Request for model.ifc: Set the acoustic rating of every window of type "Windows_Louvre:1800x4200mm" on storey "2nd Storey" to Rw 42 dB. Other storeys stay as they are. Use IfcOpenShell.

First a look at what the model holds.

```python
import ifcopenshell
import ifcopenshell.util.element

model = ifcopenshell.open("model.ifc")
print(model.schema)
storey = next(s for s in model.by_type("IfcBuildingStorey") if s.Name == "2nd Storey")
windows = [e for e in ifcopenshell.util.element.get_decomposition(storey) if e.is_a("IfcWindow")]
seen = {}
for e in windows:
    element_type = ifcopenshell.util.element.get_type(e)
    key = (element_type.Name if element_type != e and element_type else None, ifcopenshell.util.element.get_pset(e, "Pset_WindowCommon", "AcousticRating"))
    seen[key] = seen.get(key, 0) + 1
for (name, value), count in sorted(seen.items(), key=str):
    print(count, "x", name, "|", value)
```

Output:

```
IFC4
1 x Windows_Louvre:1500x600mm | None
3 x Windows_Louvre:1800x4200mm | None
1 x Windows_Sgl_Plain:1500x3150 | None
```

```python
import ifcopenshell
import ifcopenshell.api.pset
import ifcopenshell.util.element

model = ifcopenshell.open("model.ifc")

storey = next(s for s in model.by_type("IfcBuildingStorey") if s.Name == "2nd Storey")
windows = [e for e in ifcopenshell.util.element.get_decomposition(storey) if e.is_a("IfcWindow")]

count = 0
for e in windows:
    element_type = ifcopenshell.util.element.get_type(e)
    if element_type in (None, e) or element_type.Name != "Windows_Louvre:1800x4200mm":
        continue
    # add_pset returns the element's existing set when there is one.
    pset = ifcopenshell.api.pset.add_pset(model, product=e, name="Pset_WindowCommon")
    ifcopenshell.api.pset.edit_pset(model, pset=pset, properties={"AcousticRating": "Rw 42 dB"})
    count += 1

print(count, "windows updated")

model.write("model_edited.ifc")
```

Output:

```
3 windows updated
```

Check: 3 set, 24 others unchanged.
